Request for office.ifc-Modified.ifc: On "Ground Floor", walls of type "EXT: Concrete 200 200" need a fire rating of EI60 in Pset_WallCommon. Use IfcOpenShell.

First a look at what the model holds.

```python
import ifcopenshell
import ifcopenshell.util.element

model = ifcopenshell.open("office.ifc-Modified.ifc")
print(model.schema)
storey = next(s for s in model.by_type("IfcBuildingStorey") if s.Name == "Ground Floor")
walls = [e for e in ifcopenshell.util.element.get_decomposition(storey) if e.is_a("IfcWall")]
seen = {}
for e in walls:
    element_type = ifcopenshell.util.element.get_type(e)
    key = (element_type.Name if element_type != e and element_type else None, ifcopenshell.util.element.get_pset(e, "Pset_WallCommon", "FireRating"))
    seen[key] = seen.get(key, 0) + 1
for (name, value), count in sorted(seen.items(), key=str):
    print(count, "x", name, "|", value)
```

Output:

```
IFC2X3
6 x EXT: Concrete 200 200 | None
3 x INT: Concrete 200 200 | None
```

```python
import ifcopenshell
import ifcopenshell.api.pset
import ifcopenshell.util.element

model = ifcopenshell.open("office.ifc-Modified.ifc")

storey = next(s for s in model.by_type("IfcBuildingStorey") if s.Name == "Ground Floor")
walls = [e for e in ifcopenshell.util.element.get_decomposition(storey) if e.is_a("IfcWall")]

count = 0
for e in walls:
    element_type = ifcopenshell.util.element.get_type(e)
    if element_type in (None, e) or element_type.Name != "EXT: Concrete 200 200":
        continue
    # add_pset returns the element's existing set when there is one.
    pset = ifcopenshell.api.pset.add_pset(model, product=e, name="Pset_WallCommon")
    ifcopenshell.api.pset.edit_pset(model, pset=pset, properties={"FireRating": "EI60"})
    count += 1

print(count, "walls updated")

model.write("office.ifc-Modified_rev.ifc")
```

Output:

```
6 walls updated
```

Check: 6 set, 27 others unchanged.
